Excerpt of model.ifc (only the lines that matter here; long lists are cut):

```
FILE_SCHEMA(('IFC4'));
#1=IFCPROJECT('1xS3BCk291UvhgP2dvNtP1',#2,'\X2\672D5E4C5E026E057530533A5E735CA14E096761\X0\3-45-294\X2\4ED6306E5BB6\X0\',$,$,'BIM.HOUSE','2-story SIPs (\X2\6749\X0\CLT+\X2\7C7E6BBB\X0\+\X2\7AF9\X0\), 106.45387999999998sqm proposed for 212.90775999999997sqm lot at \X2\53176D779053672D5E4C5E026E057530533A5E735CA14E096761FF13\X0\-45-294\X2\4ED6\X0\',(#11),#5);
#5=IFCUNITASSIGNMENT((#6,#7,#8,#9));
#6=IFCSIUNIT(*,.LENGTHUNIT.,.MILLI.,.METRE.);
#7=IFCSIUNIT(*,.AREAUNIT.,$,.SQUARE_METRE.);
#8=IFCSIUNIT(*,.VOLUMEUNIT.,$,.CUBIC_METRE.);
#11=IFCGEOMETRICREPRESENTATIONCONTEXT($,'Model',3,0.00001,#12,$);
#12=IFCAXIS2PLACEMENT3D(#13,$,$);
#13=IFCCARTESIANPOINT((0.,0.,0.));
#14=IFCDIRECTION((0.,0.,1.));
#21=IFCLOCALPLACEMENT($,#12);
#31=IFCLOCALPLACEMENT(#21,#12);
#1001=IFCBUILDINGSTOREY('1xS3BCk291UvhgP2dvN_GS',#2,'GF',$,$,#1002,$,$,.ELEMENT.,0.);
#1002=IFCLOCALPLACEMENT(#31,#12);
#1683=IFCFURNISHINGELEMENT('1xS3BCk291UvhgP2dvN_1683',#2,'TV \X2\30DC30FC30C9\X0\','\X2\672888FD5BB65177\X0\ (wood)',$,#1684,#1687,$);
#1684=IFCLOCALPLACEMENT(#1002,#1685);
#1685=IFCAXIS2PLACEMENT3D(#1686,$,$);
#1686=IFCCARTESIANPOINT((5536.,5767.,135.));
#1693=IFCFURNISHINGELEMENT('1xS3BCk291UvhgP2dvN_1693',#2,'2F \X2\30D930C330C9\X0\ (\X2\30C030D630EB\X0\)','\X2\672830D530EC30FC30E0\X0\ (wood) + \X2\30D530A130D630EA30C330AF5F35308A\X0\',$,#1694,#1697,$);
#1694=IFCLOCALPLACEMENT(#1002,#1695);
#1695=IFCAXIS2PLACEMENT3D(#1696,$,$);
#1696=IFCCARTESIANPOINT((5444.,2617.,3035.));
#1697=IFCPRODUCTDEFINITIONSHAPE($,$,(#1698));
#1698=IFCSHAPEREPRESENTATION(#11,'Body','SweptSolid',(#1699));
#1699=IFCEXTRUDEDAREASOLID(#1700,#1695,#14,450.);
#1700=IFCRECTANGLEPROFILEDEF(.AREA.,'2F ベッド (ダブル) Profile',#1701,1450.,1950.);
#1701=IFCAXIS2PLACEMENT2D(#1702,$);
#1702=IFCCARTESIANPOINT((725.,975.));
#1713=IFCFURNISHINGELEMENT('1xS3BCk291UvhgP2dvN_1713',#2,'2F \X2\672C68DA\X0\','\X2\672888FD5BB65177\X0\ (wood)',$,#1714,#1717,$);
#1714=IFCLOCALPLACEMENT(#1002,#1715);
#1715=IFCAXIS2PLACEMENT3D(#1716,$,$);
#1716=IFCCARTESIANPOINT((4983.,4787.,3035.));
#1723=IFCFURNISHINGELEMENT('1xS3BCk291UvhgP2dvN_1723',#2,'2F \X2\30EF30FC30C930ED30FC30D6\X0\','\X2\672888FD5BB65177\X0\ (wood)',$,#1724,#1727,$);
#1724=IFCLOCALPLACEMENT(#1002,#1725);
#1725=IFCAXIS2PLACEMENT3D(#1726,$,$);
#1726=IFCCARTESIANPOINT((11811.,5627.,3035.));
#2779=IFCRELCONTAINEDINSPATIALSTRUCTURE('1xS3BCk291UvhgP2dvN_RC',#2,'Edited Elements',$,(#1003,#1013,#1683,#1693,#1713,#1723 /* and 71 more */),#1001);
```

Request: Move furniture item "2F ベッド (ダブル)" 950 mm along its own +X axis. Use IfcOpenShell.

```python
import ifcopenshell
import ifcopenshell.api.geometry
import ifcopenshell.util.placement

model = ifcopenshell.open("model.ifc")

item = model.by_guid("1xS3BCk291UvhgP2dvN_1693")
matrix = ifcopenshell.util.placement.get_local_placement(item.ObjectPlacement)
matrix[:3, 3] += matrix[:3, 0] * 950.0
ifcopenshell.api.geometry.edit_object_placement(model, product=item, matrix=matrix, is_si=False)

print(ifcopenshell.util.placement.get_local_placement(item.ObjectPlacement).round(3) + 0.0)

model.write("model_updated.ifc")
```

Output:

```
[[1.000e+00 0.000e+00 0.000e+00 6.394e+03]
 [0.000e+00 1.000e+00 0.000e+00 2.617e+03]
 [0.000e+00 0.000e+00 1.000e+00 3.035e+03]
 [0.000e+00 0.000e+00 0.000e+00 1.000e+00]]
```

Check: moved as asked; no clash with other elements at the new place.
